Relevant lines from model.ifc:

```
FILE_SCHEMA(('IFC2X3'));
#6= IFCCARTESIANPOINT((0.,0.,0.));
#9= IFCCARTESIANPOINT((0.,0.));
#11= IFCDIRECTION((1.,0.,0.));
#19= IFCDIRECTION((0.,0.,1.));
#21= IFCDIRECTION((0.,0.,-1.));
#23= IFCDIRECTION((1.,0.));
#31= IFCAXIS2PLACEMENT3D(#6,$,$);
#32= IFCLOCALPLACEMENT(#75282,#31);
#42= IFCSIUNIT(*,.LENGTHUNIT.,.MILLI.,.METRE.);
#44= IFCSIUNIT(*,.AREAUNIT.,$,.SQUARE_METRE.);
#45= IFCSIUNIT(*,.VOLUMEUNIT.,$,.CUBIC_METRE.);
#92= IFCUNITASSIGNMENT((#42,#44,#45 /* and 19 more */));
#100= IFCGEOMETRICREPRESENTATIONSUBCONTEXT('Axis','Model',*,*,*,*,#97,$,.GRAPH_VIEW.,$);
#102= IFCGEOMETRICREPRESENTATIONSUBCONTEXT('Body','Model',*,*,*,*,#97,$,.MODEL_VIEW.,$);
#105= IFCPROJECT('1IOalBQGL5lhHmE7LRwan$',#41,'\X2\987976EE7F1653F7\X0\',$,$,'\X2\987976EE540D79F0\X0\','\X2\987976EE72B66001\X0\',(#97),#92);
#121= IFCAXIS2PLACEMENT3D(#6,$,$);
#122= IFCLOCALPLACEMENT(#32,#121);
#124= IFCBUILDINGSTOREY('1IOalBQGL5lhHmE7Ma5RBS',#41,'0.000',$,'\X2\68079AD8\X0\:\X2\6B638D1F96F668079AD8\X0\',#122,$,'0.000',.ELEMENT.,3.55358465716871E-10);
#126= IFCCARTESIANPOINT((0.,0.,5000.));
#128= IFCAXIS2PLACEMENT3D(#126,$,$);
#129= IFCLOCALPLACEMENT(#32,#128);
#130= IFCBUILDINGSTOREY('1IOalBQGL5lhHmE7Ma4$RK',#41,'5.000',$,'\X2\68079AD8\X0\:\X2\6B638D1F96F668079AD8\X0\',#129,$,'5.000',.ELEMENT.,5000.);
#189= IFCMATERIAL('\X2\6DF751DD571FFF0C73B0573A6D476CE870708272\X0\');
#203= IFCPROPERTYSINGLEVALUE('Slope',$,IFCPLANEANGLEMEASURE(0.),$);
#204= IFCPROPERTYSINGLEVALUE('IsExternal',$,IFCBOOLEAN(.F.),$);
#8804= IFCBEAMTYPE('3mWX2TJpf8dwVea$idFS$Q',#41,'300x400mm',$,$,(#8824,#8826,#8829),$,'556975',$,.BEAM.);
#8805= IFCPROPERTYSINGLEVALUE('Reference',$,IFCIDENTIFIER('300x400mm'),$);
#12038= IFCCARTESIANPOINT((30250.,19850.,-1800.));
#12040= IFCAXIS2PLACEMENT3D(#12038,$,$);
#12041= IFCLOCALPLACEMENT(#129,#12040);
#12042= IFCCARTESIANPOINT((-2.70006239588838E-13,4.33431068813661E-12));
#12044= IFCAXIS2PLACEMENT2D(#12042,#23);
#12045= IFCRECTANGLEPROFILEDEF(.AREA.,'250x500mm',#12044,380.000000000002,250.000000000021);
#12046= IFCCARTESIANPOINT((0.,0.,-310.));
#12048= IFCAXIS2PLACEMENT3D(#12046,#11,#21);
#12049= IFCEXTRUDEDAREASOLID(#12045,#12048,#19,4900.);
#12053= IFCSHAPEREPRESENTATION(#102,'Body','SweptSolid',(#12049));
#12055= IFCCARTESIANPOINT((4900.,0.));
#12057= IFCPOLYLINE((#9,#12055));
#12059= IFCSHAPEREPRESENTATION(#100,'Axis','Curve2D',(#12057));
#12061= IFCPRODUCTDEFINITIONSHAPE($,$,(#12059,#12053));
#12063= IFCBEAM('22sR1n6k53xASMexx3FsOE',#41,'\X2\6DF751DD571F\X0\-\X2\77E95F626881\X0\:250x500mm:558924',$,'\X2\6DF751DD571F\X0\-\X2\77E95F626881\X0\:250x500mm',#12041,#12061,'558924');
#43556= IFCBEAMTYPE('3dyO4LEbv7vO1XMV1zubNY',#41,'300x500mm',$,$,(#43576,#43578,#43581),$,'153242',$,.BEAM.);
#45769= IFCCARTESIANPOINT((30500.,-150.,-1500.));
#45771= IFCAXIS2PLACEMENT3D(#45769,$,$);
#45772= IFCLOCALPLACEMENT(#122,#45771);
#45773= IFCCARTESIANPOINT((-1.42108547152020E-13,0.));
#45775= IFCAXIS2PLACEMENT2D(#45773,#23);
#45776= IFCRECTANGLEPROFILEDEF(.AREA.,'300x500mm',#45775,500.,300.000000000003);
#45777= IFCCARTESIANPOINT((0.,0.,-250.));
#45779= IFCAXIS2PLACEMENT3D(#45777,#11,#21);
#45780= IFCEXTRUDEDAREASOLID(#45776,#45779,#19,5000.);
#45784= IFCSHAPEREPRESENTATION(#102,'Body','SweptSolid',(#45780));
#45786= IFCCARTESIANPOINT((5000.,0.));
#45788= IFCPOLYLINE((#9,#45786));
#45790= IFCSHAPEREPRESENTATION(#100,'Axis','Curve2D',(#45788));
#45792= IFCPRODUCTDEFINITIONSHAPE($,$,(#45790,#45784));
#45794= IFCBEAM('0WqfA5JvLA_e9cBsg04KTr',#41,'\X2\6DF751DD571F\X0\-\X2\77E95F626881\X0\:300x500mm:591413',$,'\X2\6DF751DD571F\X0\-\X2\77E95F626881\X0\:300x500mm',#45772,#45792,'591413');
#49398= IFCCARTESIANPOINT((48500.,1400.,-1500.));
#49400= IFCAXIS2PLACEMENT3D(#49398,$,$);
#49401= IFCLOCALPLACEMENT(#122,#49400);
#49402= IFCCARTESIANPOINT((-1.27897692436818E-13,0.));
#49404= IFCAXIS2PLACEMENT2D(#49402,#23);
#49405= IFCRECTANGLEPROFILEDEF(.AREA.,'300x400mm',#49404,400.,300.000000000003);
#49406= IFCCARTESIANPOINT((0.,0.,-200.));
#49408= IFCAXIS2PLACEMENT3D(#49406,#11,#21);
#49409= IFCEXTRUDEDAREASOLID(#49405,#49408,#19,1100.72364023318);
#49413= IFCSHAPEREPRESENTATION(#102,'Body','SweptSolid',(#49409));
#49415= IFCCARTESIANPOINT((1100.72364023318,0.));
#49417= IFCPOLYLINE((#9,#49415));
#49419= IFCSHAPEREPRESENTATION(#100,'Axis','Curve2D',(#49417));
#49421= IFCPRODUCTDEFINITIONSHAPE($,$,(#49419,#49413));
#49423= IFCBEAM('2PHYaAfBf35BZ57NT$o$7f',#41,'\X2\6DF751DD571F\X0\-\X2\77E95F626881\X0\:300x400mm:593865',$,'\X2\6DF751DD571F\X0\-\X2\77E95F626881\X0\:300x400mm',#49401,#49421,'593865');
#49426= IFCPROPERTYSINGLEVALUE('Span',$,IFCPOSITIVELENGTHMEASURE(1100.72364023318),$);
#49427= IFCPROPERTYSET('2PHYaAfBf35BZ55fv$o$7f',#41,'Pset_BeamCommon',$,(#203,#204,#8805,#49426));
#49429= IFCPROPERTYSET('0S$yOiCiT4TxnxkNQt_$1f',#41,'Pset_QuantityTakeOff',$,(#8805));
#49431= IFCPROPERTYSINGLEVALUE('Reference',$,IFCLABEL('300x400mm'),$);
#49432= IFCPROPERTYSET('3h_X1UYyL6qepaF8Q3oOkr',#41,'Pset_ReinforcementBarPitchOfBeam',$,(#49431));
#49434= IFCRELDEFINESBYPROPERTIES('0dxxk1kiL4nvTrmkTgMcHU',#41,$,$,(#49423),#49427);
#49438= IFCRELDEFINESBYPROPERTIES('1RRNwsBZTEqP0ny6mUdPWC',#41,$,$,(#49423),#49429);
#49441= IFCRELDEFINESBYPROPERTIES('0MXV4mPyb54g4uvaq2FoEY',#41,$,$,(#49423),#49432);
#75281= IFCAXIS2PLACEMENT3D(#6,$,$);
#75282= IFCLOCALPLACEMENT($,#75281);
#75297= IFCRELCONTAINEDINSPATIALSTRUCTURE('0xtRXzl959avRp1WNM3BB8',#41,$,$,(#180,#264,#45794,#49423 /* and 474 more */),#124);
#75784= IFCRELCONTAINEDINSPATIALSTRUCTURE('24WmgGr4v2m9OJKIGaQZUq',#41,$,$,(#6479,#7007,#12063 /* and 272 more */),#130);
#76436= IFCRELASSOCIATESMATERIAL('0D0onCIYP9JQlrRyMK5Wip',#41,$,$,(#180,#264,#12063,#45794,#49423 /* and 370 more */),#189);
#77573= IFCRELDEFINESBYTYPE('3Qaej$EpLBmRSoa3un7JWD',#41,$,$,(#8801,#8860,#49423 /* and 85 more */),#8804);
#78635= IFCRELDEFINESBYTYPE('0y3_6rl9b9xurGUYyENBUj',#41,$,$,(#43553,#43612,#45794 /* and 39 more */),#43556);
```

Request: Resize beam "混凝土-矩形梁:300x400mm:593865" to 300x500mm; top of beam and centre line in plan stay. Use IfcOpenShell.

```python
import ifcopenshell
import ifcopenshell.api.pset
import ifcopenshell.api.type
import ifcopenshell.util.element
import ifcopenshell.util.representation

model = ifcopenshell.open("model.ifc")

member = model.by_id(49423)
source = next(p for p in model.by_type("IfcRectangleProfileDef") if p.ProfileName == "300x500mm")

body = ifcopenshell.util.representation.get_representation(member, "Model", "Body")
solid = body.Items[0]
old_profile = solid.SweptArea

# Copy the section's sizes but keep this member's own profile position.
profile = ifcopenshell.util.element.copy(model, source)
# Profiles are centred, so shift by half the change in depth to hold the top.
shift = (old_profile.XDim - profile.XDim) / 2
x, y = old_profile.Position.Location.Coordinates
up = (-1.0, 0.0)  # upwards, in the solid's own plane
location = model.createIfcCartesianPoint((x + up[0] * shift, y + up[1] * shift))
profile.Position = model.createIfcAxis2Placement2D(location, old_profile.Position.RefDirection)
solid.SweptArea = profile
if not model.get_total_inverses(old_profile):
    ifcopenshell.util.element.remove_deep2(model, old_profile)

new_type = model.by_id(43556)
ifcopenshell.api.type.assign_type(
    model, related_objects=[member], relating_type=new_type, should_map_representations=False
)
member.Name = member.Name.replace("300x400mm", "300x500mm")
member.ObjectType = "混凝土-矩形梁:300x500mm"
pset = model.by_id(ifcopenshell.util.element.get_pset(member, "Pset_BeamCommon", should_inherit=False)["id"])
ifcopenshell.api.pset.edit_pset(model, pset=pset, properties={"Reference": "300x500mm"})
pset = model.by_id(ifcopenshell.util.element.get_pset(member, "Pset_QuantityTakeOff", should_inherit=False)["id"])
ifcopenshell.api.pset.edit_pset(model, pset=pset, properties={"Reference": "300x500mm"})
pset = model.by_id(ifcopenshell.util.element.get_pset(member, "Pset_ReinforcementBarPitchOfBeam", should_inherit=False)["id"])
ifcopenshell.api.pset.edit_pset(model, pset=pset, properties={"Reference": "300x500mm"})

print(solid.SweptArea)

model.write("model-out.ifc")
```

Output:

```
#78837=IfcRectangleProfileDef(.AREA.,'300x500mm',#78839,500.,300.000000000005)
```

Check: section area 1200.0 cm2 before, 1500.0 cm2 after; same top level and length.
